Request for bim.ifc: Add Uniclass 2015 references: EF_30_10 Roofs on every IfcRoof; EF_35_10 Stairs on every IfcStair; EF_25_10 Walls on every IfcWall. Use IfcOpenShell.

First a look at what the model holds.

```python
import ifcopenshell

model = ifcopenshell.open("bim.ifc")
print(model.schema)
print("classifications:", [c.Name for c in model.by_type("IfcClassification")])
for ifc_class in ("IfcDoor", "IfcRoof", "IfcStair", "IfcWall", "IfcWindow"):
    print(ifc_class, len(model.by_type(ifc_class)))
```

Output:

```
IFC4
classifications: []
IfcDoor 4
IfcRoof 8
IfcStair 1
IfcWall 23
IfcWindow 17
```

```python
import ifcopenshell
import ifcopenshell.api.classification

model = ifcopenshell.open("bim.ifc")

system = ifcopenshell.api.classification.add_classification(model, classification="Uniclass 2015")

codes = {
    "IfcRoof": ("EF_30_10", "Roofs"),
    "IfcStair": ("EF_35_10", "Stairs"),
    "IfcWall": ("EF_25_10", "Walls"),
}
for ifc_class, (code, name) in codes.items():
    products = model.by_type(ifc_class)
    ifcopenshell.api.classification.add_reference(
        model, products=products, classification=system, identification=code, name=name
    )
    print(code, len(products))

model.write("bim_rev.ifc")
```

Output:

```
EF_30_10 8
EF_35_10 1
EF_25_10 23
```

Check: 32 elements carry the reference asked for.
